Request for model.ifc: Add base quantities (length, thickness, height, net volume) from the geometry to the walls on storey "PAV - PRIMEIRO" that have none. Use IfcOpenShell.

First a look at what the model holds.

```python
import ifcopenshell
import ifcopenshell.util.element
import ifcopenshell.util.unit

model = ifcopenshell.open("model.ifc")
print(model.schema)
for unit_type in ("LENGTHUNIT", "AREAUNIT", "VOLUMEUNIT"):
    print(unit_type, ifcopenshell.util.unit.calculate_unit_scale(model, unit_type))
storey = next(s for s in model.by_type("IfcBuildingStorey") if s.Name == "PAV - PRIMEIRO")
walls = [e for e in ifcopenshell.util.element.get_decomposition(storey) if e.is_a("IfcWall")]
for e in sorted(walls, key=lambda e: e.id()):
    print(e.id(), e.is_a(), e.Name, list(ifcopenshell.util.element.get_psets(e, qtos_only=True)), sep=" | ")
```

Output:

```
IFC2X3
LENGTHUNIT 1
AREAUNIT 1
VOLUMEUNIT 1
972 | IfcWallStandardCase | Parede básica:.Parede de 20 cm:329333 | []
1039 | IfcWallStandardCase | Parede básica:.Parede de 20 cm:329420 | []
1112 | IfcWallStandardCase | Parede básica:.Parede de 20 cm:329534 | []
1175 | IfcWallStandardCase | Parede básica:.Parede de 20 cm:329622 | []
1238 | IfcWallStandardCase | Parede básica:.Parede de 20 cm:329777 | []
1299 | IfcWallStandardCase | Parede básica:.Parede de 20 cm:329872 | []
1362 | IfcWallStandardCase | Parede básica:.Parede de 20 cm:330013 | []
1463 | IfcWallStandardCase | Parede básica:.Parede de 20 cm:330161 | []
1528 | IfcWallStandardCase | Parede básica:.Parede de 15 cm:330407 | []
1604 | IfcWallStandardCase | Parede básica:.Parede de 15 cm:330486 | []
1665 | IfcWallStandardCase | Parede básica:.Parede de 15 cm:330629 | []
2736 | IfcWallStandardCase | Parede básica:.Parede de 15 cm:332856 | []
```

```python
import ifcopenshell
import ifcopenshell.api.pset
import ifcopenshell.geom
import ifcopenshell.util.element
import ifcopenshell.util.shape
import ifcopenshell.util.unit

model = ifcopenshell.open("model.ifc")
unit_scale = ifcopenshell.util.unit.calculate_unit_scale(model)
volume_scale = ifcopenshell.util.unit.calculate_unit_scale(model, "VOLUMEUNIT")
settings = ifcopenshell.geom.settings()

storey = next(s for s in model.by_type("IfcBuildingStorey") if s.Name == "PAV - PRIMEIRO")
walls = [e for e in ifcopenshell.util.element.get_decomposition(storey) if e.is_a("IfcWall")]

for e in sorted(walls, key=lambda e: e.id()):
    if ifcopenshell.util.element.get_psets(e, qtos_only=True, should_inherit=False):
        continue
    # Geometry comes back in metres, in the element's own axes.
    shape = ifcopenshell.geom.create_shape(settings, e)
    values = {
        "Length": ifcopenshell.util.shape.get_x(shape.geometry) / unit_scale,
        "Width": ifcopenshell.util.shape.get_y(shape.geometry) / unit_scale,
        "Height": ifcopenshell.util.shape.get_z(shape.geometry) / unit_scale,
        "NetVolume": ifcopenshell.util.shape.get_volume(shape.geometry) / volume_scale,
    }
    qto = ifcopenshell.api.pset.add_qto(model, product=e, name="BaseQuantities")
    ifcopenshell.api.pset.edit_qto(model, qto=qto, properties=values)
    print(e.id(), {k: round(v, 3) for k, v in values.items()})

model.write("model_rev.ifc")
```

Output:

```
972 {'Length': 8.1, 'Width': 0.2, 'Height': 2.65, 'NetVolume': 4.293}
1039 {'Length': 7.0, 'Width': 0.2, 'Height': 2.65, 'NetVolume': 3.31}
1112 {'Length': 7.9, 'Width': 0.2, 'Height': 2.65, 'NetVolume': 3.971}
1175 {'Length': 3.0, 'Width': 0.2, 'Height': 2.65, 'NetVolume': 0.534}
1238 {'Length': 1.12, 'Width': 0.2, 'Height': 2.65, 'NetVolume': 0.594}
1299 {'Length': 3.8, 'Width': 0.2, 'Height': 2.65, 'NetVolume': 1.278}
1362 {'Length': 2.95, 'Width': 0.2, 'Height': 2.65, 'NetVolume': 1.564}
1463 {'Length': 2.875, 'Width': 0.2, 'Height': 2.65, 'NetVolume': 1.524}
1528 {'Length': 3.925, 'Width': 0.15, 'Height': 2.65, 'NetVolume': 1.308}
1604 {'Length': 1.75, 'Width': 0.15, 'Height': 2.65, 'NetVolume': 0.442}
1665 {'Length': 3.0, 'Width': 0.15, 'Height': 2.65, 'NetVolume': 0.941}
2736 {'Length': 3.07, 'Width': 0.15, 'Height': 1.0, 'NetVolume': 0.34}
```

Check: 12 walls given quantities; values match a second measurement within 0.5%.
